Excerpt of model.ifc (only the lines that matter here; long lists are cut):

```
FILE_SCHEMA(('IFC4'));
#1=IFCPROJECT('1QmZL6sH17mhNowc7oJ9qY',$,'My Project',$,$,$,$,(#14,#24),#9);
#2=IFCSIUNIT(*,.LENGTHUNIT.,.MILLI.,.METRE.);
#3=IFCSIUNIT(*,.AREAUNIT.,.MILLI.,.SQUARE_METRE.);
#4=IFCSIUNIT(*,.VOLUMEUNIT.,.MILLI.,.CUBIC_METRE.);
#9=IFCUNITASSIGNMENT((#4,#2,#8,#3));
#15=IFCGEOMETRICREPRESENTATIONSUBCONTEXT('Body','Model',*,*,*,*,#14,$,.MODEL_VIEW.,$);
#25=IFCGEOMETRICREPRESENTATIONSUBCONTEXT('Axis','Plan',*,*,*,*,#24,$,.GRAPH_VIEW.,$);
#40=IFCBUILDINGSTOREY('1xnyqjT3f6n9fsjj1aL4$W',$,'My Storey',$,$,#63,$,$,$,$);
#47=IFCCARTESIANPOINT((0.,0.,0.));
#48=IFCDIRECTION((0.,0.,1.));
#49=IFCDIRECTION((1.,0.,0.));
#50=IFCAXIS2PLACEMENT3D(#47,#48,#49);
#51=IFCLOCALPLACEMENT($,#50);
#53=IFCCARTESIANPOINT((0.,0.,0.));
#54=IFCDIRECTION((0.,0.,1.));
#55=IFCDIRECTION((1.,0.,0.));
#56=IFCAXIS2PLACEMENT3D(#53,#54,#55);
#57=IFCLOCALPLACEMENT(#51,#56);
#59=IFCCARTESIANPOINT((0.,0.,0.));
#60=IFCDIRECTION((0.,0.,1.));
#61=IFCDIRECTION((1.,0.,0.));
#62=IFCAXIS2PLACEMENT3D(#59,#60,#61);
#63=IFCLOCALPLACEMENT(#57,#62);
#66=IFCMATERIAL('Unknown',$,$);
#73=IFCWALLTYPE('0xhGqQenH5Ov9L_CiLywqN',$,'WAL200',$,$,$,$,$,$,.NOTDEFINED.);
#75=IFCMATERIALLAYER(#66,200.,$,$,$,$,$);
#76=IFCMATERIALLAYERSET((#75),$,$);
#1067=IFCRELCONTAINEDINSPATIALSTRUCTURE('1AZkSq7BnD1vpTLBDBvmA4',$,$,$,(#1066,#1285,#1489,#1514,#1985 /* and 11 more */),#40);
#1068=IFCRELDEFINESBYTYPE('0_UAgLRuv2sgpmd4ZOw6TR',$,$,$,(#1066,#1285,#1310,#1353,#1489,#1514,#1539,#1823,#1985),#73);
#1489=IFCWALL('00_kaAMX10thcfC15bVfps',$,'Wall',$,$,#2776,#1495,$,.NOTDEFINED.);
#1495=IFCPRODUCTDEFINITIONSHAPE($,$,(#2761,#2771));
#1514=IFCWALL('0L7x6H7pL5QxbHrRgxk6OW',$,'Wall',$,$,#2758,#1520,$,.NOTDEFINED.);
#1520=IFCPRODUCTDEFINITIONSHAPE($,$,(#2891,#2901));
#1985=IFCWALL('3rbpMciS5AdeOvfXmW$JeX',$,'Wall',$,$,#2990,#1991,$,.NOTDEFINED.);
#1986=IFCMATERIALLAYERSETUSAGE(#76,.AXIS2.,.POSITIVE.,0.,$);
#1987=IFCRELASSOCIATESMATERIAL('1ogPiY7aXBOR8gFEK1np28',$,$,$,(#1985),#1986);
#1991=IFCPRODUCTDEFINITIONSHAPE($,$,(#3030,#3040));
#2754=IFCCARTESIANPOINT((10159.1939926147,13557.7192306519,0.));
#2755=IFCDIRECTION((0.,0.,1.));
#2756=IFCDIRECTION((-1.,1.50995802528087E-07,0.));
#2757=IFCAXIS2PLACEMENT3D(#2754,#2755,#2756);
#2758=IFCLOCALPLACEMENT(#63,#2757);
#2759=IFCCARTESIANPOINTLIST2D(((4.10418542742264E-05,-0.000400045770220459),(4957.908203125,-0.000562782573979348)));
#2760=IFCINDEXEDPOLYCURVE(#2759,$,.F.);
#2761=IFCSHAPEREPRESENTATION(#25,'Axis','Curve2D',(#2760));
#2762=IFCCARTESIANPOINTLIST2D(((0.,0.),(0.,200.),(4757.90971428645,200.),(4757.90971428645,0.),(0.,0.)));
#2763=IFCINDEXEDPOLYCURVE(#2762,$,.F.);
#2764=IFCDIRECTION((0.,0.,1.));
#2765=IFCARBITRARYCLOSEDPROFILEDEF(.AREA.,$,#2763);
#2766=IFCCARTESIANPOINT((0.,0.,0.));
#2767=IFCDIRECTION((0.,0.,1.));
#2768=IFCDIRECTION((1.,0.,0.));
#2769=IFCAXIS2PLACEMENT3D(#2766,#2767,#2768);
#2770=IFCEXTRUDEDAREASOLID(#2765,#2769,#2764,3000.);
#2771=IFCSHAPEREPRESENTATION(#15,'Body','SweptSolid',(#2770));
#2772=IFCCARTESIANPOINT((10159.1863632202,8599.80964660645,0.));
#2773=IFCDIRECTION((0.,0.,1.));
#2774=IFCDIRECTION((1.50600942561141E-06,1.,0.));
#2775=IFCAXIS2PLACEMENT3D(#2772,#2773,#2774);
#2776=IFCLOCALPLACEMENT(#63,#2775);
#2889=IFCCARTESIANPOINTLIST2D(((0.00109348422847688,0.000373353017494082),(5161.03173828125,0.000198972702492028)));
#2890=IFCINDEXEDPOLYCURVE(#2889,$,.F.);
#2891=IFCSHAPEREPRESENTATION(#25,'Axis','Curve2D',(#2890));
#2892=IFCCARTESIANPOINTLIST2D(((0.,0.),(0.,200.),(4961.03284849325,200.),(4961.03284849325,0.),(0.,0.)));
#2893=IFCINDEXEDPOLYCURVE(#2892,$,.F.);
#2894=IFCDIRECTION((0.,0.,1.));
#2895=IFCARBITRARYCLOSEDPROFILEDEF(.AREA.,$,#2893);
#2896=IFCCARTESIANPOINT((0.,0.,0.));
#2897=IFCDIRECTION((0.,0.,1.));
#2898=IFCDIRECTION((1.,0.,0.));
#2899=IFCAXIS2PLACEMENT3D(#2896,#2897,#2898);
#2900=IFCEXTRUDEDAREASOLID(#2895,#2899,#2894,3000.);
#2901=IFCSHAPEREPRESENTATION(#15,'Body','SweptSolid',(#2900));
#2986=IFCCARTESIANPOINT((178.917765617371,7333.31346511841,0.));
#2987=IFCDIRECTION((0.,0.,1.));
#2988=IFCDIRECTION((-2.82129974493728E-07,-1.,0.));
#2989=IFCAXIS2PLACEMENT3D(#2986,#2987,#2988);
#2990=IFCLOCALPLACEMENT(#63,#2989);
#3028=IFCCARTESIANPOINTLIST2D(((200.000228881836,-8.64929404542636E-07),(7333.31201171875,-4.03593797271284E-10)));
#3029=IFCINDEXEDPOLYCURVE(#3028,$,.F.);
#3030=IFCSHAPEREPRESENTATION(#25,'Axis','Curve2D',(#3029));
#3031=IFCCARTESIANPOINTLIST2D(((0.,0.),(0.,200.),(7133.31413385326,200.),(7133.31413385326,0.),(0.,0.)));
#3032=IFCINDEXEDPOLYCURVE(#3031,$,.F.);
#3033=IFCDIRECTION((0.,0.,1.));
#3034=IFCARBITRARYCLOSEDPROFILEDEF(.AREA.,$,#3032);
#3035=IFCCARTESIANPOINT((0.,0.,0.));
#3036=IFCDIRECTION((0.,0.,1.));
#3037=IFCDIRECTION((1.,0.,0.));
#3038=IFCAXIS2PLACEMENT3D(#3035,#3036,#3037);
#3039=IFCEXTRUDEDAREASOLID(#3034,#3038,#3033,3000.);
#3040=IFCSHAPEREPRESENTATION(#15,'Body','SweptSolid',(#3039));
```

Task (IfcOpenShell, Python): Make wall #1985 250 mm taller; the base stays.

```python
import ifcopenshell
import ifcopenshell.geom
import ifcopenshell.util.representation
import ifcopenshell.util.shape
import ifcopenshell.util.unit

model = ifcopenshell.open("model.ifc")
unit_scale = ifcopenshell.util.unit.calculate_unit_scale(model)
settings = ifcopenshell.geom.settings()


def volume(element):
    """Net volume in cubic metres, openings subtracted."""
    shape = ifcopenshell.geom.create_shape(settings, element)
    return ifcopenshell.util.shape.get_volume(shape.geometry)


wall = model.by_guid("3rbpMciS5AdeOvfXmW$JeX")
before = volume(wall)

body = ifcopenshell.util.representation.get_representation(wall, "Model", "Body")
solid = body.Items[0]
old_height = solid.Depth
solid.Depth += 0.25 / unit_scale
after = volume(wall)

print(f"height {old_height:g} -> {solid.Depth:g}, volume {before:.3f} -> {after:.3f} m3")

model.write("model_edited.ifc")
```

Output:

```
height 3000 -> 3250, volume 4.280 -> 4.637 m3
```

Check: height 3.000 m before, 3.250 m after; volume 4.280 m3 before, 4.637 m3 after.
